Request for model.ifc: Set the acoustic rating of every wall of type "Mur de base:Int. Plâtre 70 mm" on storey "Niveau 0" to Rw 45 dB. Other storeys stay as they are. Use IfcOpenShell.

First a look at what the model holds.

```python
import ifcopenshell
import ifcopenshell.util.element

model = ifcopenshell.open("model.ifc")
print(model.schema)
storey = next(s for s in model.by_type("IfcBuildingStorey") if s.Name == "Niveau 0")
walls = [e for e in ifcopenshell.util.element.get_decomposition(storey) if e.is_a("IfcWall")]
seen = {}
for e in walls:
    element_type = ifcopenshell.util.element.get_type(e)
    key = (element_type.Name if element_type != e and element_type else None, ifcopenshell.util.element.get_pset(e, "Pset_WallCommon", "AcousticRating"))
    seen[key] = seen.get(key, 0) + 1
for (name, value), count in sorted(seen.items(), key=str):
    print(count, "x", name, "|", value)
```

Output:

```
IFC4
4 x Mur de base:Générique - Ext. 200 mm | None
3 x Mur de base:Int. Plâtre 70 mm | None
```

```python
import ifcopenshell
import ifcopenshell.api.pset
import ifcopenshell.util.element

model = ifcopenshell.open("model.ifc")

storey = next(s for s in model.by_type("IfcBuildingStorey") if s.Name == "Niveau 0")
walls = [e for e in ifcopenshell.util.element.get_decomposition(storey) if e.is_a("IfcWall")]

count = 0
for e in walls:
    element_type = ifcopenshell.util.element.get_type(e)
    if element_type in (None, e) or element_type.Name != "Mur de base:Int. Plâtre 70 mm":
        continue
    # add_pset returns the element's existing set when there is one.
    pset = ifcopenshell.api.pset.add_pset(model, product=e, name="Pset_WallCommon")
    ifcopenshell.api.pset.edit_pset(model, pset=pset, properties={"AcousticRating": "Rw 45 dB"})
    count += 1

print(count, "walls updated")

model.write("model_v2.ifc")
```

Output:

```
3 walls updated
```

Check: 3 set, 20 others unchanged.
